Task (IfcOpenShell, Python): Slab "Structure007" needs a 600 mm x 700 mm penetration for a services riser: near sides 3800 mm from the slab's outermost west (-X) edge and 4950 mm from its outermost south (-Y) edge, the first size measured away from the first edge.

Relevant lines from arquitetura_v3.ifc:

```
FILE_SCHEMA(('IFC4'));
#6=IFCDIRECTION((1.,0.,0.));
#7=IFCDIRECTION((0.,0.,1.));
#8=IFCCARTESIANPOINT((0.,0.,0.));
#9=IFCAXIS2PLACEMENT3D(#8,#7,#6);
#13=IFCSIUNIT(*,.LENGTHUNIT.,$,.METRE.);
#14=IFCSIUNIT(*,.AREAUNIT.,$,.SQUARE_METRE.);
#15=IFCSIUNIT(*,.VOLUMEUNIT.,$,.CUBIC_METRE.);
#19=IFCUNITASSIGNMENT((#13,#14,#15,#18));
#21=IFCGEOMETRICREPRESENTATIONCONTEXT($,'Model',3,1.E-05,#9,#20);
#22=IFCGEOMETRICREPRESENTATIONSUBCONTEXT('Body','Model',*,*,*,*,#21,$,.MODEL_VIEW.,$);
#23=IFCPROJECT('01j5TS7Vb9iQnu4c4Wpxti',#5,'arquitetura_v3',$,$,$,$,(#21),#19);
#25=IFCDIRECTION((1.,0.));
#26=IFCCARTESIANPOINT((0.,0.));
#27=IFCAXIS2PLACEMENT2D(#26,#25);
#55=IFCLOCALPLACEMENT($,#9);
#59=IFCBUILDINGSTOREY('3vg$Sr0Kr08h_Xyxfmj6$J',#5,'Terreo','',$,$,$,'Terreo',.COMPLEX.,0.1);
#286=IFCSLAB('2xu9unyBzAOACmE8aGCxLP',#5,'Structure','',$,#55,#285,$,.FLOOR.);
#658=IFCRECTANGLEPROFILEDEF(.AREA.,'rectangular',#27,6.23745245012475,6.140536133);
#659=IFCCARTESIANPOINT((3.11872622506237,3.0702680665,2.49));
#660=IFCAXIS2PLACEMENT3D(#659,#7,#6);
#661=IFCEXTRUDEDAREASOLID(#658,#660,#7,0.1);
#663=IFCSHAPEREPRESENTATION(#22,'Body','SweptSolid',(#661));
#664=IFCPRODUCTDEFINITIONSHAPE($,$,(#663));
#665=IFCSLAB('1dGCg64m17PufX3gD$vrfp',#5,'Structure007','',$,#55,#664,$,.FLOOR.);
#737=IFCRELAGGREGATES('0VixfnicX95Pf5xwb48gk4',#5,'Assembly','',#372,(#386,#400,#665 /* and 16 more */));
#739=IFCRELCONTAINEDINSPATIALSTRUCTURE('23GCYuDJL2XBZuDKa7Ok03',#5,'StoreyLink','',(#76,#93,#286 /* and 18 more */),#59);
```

```python
import numpy as np
import ifcopenshell
import ifcopenshell.api.feature
import ifcopenshell.api.geometry
import ifcopenshell.api.root
import ifcopenshell.geom
import ifcopenshell.util.placement
import ifcopenshell.util.representation
import ifcopenshell.util.shape
import ifcopenshell.util.unit

model = ifcopenshell.open("arquitetura_v3.ifc")
unit_scale = ifcopenshell.util.unit.calculate_unit_scale(model)
settings = ifcopenshell.geom.settings()


def volume(element):
    """Net volume in cubic metres, openings subtracted."""
    shape = ifcopenshell.geom.create_shape(settings, element)
    return ifcopenshell.util.shape.get_volume(shape.geometry)


slab = model.by_guid("1dGCg64m17PufX3gD$vrfp")
before = volume(slab)

# Extent in the slab's own axes, in metres. The edges named are its -X and -Y sides.
slab_shape = ifcopenshell.geom.create_shape(settings, slab)
vertices = ifcopenshell.util.shape.get_vertices(slab_shape.geometry)
x_min, y_min, bottom = vertices.min(axis=0)
top = vertices[:, 2].max()

opening = ifcopenshell.api.root.create_entity(model, ifc_class="IfcOpeningElement", name="Services riser opening", predefined_type="OPENING")
context = ifcopenshell.util.representation.get_context(model, "Model", "Body", "MODEL_VIEW")
width, depth = 0.6, 0.7
outline = [(0.0, 0.0), (width, 0.0), (width, depth), (0.0, depth), (0.0, 0.0)]
# Overshoot both faces by 50 mm so the cut is clean.
shape = ifcopenshell.api.geometry.add_slab_representation(
    model, context=context, depth=top - bottom + 0.1, polyline=outline
)
ifcopenshell.api.geometry.assign_representation(model, product=opening, representation=shape)

matrix = ifcopenshell.util.placement.get_local_placement(slab.ObjectPlacement)
matrix[:, 3] = matrix @ np.append(np.array([x_min + 3.8, y_min + 4.95, bottom - 0.05]) / unit_scale, 1.0)
ifcopenshell.api.geometry.edit_object_placement(model, product=opening, matrix=matrix, is_si=False)
ifcopenshell.api.feature.add_feature(model, feature=opening, element=slab)

after = volume(slab)

print(f"slab volume {before:.3f} -> {after:.3f} m3")

model.write("arquitetura_v3_edited.ifc")
```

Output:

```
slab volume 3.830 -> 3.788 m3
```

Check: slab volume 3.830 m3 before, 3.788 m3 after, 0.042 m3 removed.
